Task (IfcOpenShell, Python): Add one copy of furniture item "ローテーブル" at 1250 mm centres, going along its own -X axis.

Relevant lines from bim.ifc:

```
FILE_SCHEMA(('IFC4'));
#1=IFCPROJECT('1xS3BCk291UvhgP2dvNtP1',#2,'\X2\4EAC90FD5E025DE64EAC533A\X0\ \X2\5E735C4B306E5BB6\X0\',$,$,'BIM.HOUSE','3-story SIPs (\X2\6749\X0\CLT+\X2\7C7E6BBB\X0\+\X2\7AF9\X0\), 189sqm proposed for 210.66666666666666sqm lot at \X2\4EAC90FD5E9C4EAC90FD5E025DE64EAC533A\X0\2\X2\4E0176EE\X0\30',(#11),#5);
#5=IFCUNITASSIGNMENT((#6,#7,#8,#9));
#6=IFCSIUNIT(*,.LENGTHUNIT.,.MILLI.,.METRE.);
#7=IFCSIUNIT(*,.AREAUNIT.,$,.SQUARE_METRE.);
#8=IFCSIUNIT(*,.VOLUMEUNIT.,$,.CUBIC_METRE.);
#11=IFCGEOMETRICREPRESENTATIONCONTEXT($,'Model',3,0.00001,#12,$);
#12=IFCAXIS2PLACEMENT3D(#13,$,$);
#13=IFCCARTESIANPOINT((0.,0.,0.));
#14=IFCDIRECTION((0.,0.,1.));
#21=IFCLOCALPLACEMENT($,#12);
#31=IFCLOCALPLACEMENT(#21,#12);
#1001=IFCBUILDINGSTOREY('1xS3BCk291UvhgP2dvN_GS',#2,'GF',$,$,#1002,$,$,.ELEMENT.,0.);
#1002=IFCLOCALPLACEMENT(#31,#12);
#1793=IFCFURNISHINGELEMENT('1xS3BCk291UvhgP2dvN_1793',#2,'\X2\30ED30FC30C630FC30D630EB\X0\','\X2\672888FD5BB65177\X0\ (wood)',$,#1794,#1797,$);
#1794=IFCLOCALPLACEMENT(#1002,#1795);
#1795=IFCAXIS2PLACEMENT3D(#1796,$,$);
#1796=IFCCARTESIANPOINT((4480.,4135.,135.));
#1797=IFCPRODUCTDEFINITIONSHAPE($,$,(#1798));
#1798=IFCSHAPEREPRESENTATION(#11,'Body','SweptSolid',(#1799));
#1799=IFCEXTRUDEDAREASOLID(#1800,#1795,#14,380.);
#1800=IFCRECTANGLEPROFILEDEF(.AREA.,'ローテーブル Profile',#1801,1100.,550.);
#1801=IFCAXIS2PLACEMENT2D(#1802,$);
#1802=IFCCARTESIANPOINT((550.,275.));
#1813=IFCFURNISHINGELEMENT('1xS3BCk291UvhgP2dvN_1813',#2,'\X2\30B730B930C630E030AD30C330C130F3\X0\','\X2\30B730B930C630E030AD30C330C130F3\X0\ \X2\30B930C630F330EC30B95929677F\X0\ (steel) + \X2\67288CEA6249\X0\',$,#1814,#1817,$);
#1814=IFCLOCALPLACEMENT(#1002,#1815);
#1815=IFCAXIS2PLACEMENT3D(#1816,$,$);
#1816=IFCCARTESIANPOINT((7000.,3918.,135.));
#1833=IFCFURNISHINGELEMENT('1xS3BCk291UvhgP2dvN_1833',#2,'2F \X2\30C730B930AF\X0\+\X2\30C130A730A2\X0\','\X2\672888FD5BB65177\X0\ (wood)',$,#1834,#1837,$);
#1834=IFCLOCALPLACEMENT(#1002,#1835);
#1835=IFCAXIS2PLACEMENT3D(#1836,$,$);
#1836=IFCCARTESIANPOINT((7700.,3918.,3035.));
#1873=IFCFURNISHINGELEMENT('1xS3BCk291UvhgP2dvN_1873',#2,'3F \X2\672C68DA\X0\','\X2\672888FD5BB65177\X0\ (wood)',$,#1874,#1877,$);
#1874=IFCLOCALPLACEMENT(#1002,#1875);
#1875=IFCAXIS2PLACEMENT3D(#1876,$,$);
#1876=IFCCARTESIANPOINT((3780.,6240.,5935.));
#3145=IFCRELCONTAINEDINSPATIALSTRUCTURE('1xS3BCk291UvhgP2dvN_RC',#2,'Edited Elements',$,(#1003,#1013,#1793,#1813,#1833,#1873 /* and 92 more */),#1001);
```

```python
import ifcopenshell
import ifcopenshell.api.geometry
import ifcopenshell.api.root
import ifcopenshell.util.element
import ifcopenshell.util.placement

model = ifcopenshell.open("bim.ifc")


def reuse_history(source, copy):
    """copy_class also copies each property set's owner history, people and application; keep the originals."""
    for rel in copy.IsDefinedBy:
        if rel.is_a("IfcRelDefinesByProperties") and (history := rel.RelatingPropertyDefinition.OwnerHistory):
            rel.RelatingPropertyDefinition.OwnerHistory = source.OwnerHistory
            ifcopenshell.util.element.remove_deep2(model, history)


source = model.by_guid("1xS3BCk291UvhgP2dvN_1793")
base = ifcopenshell.util.placement.get_local_placement(source.ObjectPlacement)
step = -base[:3, 0] * 1250.0

for i in range(1, 2):
    copy = ifcopenshell.api.root.copy_class(model, product=source)
    copy.Representation = ifcopenshell.util.element.copy_deep(
        model, source.Representation, exclude=["IfcGeometricRepresentationContext", "IfcRepresentationMap"]
    )
    reuse_history(source, copy)
    matrix = base.copy()
    matrix[:3, 3] += i * step
    print("added at", matrix[:3, 3].round(3) + 0.0)
    ifcopenshell.api.geometry.edit_object_placement(model, product=copy, matrix=matrix, is_si=False)

model.write("bim_edited.ifc")
```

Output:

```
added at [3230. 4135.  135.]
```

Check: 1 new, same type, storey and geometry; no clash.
